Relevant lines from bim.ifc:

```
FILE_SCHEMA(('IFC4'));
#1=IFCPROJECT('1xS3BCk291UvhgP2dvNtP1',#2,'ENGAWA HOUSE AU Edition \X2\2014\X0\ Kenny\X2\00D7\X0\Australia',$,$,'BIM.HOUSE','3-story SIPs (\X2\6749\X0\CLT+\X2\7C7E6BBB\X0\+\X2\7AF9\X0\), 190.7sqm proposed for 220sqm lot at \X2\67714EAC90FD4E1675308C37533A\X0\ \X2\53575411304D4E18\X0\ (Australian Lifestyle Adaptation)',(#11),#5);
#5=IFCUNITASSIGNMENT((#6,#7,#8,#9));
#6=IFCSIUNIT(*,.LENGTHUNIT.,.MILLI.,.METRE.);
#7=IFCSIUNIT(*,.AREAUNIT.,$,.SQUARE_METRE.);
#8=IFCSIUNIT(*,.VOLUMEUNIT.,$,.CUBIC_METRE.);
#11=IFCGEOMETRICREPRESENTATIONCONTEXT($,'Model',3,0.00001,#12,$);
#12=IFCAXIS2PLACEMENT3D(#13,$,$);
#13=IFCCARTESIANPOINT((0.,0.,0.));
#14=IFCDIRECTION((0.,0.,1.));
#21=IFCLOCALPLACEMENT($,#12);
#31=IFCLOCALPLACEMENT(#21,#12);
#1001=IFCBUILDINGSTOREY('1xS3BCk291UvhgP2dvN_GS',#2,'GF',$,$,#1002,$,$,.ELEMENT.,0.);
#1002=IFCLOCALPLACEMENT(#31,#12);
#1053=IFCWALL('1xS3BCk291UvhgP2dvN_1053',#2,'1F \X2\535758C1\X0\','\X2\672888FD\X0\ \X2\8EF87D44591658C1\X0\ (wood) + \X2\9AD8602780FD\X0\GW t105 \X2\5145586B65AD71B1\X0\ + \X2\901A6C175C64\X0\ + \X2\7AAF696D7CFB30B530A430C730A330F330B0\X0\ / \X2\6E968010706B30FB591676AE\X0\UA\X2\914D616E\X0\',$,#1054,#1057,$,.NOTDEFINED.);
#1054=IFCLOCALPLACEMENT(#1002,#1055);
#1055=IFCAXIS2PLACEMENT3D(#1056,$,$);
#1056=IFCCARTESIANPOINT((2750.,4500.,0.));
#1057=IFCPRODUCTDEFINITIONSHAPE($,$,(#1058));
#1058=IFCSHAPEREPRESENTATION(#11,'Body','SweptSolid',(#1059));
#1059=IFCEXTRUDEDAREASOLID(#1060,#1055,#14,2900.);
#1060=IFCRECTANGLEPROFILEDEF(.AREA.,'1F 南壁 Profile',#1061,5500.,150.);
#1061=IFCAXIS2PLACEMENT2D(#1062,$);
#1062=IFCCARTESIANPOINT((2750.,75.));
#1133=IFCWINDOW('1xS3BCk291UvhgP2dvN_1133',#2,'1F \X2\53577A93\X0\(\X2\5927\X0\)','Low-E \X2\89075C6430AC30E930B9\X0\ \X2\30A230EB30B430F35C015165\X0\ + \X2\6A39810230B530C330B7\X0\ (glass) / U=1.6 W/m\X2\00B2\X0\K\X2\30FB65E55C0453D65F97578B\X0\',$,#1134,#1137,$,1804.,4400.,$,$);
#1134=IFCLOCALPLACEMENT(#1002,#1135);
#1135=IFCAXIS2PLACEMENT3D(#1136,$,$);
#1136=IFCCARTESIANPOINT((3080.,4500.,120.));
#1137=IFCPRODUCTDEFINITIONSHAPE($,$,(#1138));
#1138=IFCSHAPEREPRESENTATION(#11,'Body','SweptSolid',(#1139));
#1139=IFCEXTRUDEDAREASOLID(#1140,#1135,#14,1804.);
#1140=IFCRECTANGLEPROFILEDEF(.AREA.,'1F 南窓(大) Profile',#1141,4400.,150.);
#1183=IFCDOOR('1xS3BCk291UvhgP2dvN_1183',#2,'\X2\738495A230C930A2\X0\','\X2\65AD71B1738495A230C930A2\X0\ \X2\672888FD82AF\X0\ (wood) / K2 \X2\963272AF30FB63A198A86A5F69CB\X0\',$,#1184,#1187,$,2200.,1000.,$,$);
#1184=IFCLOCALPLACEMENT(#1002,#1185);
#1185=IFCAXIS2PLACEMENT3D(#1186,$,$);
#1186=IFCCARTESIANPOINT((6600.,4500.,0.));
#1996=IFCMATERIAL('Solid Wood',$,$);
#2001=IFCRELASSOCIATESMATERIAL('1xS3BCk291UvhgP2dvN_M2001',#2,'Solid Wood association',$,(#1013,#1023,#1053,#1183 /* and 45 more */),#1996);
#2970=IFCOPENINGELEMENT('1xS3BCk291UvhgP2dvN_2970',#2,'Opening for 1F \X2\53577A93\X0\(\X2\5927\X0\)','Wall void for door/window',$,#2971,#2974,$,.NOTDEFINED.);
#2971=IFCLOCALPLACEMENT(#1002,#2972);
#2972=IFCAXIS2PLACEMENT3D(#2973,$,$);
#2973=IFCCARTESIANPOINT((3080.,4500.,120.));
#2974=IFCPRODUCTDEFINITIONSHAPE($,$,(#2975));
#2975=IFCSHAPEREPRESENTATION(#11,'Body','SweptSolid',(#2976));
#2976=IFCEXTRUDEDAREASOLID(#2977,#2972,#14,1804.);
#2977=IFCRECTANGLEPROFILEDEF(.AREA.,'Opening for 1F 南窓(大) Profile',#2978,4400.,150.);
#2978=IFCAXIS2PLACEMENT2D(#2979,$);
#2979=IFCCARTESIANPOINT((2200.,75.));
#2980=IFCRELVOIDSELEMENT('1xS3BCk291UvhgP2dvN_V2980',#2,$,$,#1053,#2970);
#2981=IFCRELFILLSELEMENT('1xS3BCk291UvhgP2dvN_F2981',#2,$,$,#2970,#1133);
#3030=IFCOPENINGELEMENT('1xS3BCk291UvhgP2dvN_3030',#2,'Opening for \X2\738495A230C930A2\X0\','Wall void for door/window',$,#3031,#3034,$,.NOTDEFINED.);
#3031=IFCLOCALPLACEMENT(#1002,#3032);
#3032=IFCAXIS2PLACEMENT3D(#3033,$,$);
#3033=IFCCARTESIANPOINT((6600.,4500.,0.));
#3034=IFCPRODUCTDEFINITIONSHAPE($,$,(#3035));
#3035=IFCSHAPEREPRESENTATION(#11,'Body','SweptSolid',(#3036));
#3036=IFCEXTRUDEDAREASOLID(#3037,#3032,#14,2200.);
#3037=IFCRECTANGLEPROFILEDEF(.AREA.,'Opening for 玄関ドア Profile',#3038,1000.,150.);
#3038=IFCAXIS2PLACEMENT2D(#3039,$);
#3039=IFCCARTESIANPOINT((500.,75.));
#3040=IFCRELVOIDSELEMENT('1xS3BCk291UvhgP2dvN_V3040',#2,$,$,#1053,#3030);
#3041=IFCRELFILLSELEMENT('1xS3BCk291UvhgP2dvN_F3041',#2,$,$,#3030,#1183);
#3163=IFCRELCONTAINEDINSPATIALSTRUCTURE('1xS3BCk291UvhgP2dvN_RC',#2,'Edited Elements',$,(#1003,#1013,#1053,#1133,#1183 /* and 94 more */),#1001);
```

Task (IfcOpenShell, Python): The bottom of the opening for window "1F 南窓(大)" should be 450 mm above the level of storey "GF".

```python
import numpy as np
import ifcopenshell
import ifcopenshell.api.geometry
import ifcopenshell.geom
import ifcopenshell.util.element
import ifcopenshell.util.placement
import ifcopenshell.util.shape
import ifcopenshell.util.unit

model = ifcopenshell.open("bim.ifc")
unit_scale = ifcopenshell.util.unit.calculate_unit_scale(model)

window = model.by_guid("1xS3BCk291UvhgP2dvN_1133")
opening = window.FillsVoids[0].RelatingOpeningElement
storey = ifcopenshell.util.element.get_container(window, ifc_class="IfcBuildingStorey")
level = ifcopenshell.util.placement.get_local_placement(storey.ObjectPlacement)[2, 3]

# The opening's origin need not be at the sill, so measure its lowest point.
shape = ifcopenshell.geom.create_shape(ifcopenshell.geom.settings(), opening)
bottom = ifcopenshell.util.shape.get_shape_bottom_elevation(shape, shape.geometry) / unit_scale
dz = level + 450.0 - bottom

shift = np.array([0.0, 0.0, dz])
# The window is not placed relative to its opening, so move both.
for product in (opening, window):
    matrix = ifcopenshell.util.placement.get_local_placement(product.ObjectPlacement)
    matrix[:3, 3] += shift
    ifcopenshell.api.geometry.edit_object_placement(model, product=product, matrix=matrix, is_si=False)

print(f"moved by {dz * unit_scale:+.3f} m")

model.write("bim-out.ifc")
```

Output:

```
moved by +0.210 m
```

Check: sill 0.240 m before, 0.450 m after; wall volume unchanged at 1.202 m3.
